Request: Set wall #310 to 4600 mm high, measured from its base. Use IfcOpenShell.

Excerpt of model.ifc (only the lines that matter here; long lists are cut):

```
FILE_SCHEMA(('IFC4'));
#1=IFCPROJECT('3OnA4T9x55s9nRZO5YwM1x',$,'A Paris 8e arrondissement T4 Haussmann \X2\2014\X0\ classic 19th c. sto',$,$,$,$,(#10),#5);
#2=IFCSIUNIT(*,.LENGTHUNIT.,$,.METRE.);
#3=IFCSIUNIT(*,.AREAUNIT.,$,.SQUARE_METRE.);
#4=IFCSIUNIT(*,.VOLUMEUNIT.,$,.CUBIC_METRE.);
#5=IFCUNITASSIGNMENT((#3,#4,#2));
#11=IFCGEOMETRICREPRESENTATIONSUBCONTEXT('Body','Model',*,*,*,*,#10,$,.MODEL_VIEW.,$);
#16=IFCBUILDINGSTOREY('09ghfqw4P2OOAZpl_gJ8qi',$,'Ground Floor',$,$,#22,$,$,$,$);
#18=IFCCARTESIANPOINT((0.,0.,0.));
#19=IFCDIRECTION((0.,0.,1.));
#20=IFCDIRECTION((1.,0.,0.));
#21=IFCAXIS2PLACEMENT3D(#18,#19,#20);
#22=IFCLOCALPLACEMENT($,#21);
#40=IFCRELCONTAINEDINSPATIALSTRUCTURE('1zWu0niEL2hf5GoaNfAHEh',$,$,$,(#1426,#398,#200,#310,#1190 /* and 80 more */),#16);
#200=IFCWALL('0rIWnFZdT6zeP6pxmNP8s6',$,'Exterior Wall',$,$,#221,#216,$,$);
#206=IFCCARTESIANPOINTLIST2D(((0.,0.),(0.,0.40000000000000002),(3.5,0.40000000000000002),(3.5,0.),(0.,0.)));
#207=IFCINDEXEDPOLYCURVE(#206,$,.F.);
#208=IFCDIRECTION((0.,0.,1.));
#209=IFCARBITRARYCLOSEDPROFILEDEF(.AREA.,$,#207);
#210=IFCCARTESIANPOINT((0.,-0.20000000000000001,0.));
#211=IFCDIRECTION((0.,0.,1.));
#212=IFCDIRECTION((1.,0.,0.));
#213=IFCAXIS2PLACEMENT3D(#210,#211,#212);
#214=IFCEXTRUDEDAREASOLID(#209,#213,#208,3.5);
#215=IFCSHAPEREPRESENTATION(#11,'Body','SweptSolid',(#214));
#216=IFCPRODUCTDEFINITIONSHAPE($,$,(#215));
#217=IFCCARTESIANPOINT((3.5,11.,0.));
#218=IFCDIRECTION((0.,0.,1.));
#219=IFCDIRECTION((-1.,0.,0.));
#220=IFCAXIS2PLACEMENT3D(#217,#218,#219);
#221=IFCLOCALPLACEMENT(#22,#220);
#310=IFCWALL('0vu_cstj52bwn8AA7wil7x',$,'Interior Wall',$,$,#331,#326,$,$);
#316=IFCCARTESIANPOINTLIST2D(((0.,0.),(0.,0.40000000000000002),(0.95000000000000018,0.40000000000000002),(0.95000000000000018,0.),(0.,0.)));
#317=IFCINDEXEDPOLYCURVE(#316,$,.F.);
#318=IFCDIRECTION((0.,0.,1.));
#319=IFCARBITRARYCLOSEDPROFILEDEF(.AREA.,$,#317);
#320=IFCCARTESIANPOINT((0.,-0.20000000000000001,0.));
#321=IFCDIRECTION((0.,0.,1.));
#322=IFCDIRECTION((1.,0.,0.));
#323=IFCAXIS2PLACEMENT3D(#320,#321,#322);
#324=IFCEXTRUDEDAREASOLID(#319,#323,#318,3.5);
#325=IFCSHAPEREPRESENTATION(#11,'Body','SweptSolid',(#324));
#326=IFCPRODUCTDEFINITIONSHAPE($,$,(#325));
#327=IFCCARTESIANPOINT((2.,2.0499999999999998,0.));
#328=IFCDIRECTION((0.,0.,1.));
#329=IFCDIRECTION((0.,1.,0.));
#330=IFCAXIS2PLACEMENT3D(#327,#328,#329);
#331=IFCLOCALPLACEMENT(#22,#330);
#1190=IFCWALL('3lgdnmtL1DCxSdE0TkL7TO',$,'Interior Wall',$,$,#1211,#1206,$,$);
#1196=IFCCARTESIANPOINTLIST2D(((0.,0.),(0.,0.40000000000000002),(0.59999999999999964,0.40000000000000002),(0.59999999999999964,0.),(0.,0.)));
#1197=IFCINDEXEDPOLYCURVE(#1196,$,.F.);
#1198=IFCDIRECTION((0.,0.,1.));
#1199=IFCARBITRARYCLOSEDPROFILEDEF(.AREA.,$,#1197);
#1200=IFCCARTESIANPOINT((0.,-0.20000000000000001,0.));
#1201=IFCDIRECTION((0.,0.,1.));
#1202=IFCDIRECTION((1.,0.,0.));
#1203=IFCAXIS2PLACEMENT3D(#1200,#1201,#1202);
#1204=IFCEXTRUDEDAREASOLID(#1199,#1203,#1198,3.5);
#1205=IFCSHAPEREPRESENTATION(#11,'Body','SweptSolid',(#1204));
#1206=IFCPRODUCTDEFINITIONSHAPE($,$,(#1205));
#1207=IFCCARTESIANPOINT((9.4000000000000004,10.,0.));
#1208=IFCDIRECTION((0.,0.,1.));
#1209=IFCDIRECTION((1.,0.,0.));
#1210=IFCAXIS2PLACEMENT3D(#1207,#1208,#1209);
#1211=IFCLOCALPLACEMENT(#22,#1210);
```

```python
import ifcopenshell
import ifcopenshell.geom
import ifcopenshell.util.representation
import ifcopenshell.util.shape

model = ifcopenshell.open("model.ifc")
settings = ifcopenshell.geom.settings()


def volume(element):
    """Net volume in cubic metres, openings subtracted."""
    shape = ifcopenshell.geom.create_shape(settings, element)
    return ifcopenshell.util.shape.get_volume(shape.geometry)


wall = model.by_guid("0vu_cstj52bwn8AA7wil7x")
before = volume(wall)

body = ifcopenshell.util.representation.get_representation(wall, "Model", "Body")
solid = body.Items[0]
old_height = solid.Depth
solid.Depth = 4.6
after = volume(wall)

print(f"height {old_height:g} -> {solid.Depth:g}, volume {before:.3f} -> {after:.3f} m3")

model.write("model_edited.ifc")
```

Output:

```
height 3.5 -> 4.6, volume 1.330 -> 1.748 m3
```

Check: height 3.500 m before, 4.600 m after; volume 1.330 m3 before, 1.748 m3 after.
